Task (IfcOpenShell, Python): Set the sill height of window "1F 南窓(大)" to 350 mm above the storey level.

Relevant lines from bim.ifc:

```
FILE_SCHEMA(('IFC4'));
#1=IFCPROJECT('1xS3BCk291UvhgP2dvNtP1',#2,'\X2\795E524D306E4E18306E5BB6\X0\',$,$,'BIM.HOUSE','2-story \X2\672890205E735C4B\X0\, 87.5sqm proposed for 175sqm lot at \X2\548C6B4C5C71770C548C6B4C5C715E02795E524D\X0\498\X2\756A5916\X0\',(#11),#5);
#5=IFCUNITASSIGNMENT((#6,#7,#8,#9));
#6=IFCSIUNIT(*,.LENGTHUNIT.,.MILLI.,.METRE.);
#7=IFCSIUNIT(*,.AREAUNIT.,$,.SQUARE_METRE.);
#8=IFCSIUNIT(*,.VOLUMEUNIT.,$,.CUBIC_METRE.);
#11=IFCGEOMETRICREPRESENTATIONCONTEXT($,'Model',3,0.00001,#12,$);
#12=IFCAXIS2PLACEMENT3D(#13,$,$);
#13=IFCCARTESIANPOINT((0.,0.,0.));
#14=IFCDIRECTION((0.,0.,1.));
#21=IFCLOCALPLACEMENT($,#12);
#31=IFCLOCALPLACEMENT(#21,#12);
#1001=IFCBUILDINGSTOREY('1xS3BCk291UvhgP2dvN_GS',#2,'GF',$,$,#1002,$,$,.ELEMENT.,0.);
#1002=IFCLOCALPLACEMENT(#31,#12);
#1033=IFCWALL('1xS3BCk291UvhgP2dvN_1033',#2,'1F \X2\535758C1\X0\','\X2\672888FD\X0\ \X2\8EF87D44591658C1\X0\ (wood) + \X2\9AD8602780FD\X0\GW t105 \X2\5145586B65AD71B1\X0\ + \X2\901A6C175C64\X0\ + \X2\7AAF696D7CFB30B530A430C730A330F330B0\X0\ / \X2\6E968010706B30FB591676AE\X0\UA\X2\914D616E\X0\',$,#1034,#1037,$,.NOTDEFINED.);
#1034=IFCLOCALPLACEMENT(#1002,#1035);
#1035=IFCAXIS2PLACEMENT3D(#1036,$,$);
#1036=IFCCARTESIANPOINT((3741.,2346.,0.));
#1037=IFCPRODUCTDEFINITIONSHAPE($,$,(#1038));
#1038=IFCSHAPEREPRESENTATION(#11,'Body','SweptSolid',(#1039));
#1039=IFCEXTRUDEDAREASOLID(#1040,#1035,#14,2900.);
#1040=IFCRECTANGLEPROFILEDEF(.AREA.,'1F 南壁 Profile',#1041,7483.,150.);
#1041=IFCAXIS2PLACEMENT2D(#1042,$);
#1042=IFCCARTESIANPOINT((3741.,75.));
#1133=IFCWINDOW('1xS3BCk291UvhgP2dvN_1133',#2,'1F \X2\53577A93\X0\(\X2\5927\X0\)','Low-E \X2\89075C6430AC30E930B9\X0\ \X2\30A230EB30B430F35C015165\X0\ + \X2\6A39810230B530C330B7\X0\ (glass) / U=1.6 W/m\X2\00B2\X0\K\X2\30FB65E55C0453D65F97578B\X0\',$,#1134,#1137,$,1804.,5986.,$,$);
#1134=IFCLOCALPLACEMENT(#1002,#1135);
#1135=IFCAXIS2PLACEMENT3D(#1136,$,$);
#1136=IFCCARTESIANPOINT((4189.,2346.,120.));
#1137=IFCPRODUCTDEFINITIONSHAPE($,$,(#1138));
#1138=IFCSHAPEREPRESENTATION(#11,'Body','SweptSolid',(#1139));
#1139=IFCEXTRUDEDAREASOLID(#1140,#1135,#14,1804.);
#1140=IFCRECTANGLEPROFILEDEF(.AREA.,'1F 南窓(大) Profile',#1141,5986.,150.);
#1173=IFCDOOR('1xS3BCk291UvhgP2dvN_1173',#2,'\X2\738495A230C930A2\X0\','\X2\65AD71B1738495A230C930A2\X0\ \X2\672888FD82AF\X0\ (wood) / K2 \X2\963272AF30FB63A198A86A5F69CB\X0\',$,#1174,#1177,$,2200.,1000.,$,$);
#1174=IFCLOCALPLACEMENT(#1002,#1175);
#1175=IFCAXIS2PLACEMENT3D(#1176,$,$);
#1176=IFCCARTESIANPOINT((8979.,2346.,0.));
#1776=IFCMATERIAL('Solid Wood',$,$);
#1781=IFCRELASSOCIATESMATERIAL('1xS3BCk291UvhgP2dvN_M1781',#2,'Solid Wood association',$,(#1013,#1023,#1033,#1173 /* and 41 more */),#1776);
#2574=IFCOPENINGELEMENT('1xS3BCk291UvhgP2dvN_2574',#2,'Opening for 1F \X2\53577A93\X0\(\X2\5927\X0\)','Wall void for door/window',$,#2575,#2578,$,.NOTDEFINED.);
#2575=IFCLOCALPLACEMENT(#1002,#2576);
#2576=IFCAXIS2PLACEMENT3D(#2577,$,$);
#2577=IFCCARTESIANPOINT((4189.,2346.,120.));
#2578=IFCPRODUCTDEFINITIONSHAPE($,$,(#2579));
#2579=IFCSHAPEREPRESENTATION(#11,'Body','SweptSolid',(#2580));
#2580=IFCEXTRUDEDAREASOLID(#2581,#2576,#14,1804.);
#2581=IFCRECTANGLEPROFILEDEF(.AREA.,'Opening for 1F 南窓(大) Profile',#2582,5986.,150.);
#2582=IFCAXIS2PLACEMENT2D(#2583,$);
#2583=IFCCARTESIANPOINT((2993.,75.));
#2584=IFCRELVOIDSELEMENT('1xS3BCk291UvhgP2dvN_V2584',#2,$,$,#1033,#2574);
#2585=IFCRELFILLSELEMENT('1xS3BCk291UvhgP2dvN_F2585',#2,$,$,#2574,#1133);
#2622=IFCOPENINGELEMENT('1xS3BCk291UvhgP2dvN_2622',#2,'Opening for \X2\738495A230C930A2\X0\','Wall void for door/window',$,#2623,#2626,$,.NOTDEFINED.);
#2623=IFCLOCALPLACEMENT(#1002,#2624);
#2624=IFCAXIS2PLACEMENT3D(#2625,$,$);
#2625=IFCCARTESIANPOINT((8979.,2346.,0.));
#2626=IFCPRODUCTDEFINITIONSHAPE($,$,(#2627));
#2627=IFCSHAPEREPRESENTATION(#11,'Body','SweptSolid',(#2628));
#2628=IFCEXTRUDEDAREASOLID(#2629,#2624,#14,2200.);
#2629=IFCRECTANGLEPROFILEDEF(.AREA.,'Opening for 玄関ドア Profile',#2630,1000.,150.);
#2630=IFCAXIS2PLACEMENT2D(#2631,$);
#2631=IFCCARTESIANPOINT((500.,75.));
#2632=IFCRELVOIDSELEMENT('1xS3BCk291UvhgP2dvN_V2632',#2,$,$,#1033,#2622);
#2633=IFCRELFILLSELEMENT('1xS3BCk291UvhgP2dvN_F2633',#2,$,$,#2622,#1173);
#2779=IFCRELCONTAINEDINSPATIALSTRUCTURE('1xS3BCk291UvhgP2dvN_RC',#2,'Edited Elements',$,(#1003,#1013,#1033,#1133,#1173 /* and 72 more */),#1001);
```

```python
import numpy as np
import ifcopenshell
import ifcopenshell.api.geometry
import ifcopenshell.geom
import ifcopenshell.util.element
import ifcopenshell.util.placement
import ifcopenshell.util.shape
import ifcopenshell.util.unit

model = ifcopenshell.open("bim.ifc")
unit_scale = ifcopenshell.util.unit.calculate_unit_scale(model)

window = model.by_id(1133)
opening = window.FillsVoids[0].RelatingOpeningElement
storey = ifcopenshell.util.element.get_container(window, ifc_class="IfcBuildingStorey")
level = ifcopenshell.util.placement.get_local_placement(storey.ObjectPlacement)[2, 3]

# The opening's origin need not be at the sill, so measure its lowest point.
shape = ifcopenshell.geom.create_shape(ifcopenshell.geom.settings(), opening)
bottom = ifcopenshell.util.shape.get_shape_bottom_elevation(shape, shape.geometry) / unit_scale
dz = level + 0.35 / unit_scale - bottom

shift = np.array([0.0, 0.0, dz])
# The window is not placed relative to its opening, so move both.
for product in (opening, window):
    matrix = ifcopenshell.util.placement.get_local_placement(product.ObjectPlacement)
    matrix[:3, 3] += shift
    ifcopenshell.api.geometry.edit_object_placement(model, product=product, matrix=matrix, is_si=False)

print(f"moved by {dz * unit_scale:+.3f} m")

model.write("bim_updated.ifc")
```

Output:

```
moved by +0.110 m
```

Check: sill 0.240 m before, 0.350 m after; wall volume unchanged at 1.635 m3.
